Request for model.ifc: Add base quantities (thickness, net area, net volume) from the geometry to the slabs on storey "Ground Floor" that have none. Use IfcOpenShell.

First a look at what the model holds.

```python
import ifcopenshell
import ifcopenshell.util.element
import ifcopenshell.util.unit

model = ifcopenshell.open("model.ifc")
print(model.schema)
for unit_type in ("LENGTHUNIT", "AREAUNIT", "VOLUMEUNIT"):
    print(unit_type, ifcopenshell.util.unit.calculate_unit_scale(model, unit_type))
storey = next(s for s in model.by_type("IfcBuildingStorey") if s.Name == "Ground Floor")
slabs = [e for e in ifcopenshell.util.element.get_decomposition(storey) if e.is_a("IfcSlab")]
for e in sorted(slabs, key=lambda e: e.id()):
    print(e.id(), e.is_a(), e.Name, list(ifcopenshell.util.element.get_psets(e, qtos_only=True)), sep=" | ")
```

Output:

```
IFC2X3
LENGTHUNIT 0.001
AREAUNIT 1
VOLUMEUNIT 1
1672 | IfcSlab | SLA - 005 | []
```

```python
import ifcopenshell
import ifcopenshell.api.pset
import ifcopenshell.geom
import ifcopenshell.util.element
import ifcopenshell.util.shape
import ifcopenshell.util.unit

model = ifcopenshell.open("model.ifc")
unit_scale = ifcopenshell.util.unit.calculate_unit_scale(model)
area_scale = ifcopenshell.util.unit.calculate_unit_scale(model, "AREAUNIT")
volume_scale = ifcopenshell.util.unit.calculate_unit_scale(model, "VOLUMEUNIT")
settings = ifcopenshell.geom.settings()

storey = next(s for s in model.by_type("IfcBuildingStorey") if s.Name == "Ground Floor")
slabs = [e for e in ifcopenshell.util.element.get_decomposition(storey) if e.is_a("IfcSlab")]

for e in sorted(slabs, key=lambda e: e.id()):
    if ifcopenshell.util.element.get_psets(e, qtos_only=True, should_inherit=False):
        continue
    # Geometry comes back in metres, in the element's own axes.
    shape = ifcopenshell.geom.create_shape(settings, e)
    values = {
        "Width": ifcopenshell.util.shape.get_z(shape.geometry) / unit_scale,
        "NetArea": ifcopenshell.util.shape.get_footprint_area(shape.geometry) / area_scale,
        "NetVolume": ifcopenshell.util.shape.get_volume(shape.geometry) / volume_scale,
    }
    qto = ifcopenshell.api.pset.add_qto(model, product=e, name="BaseQuantities")
    ifcopenshell.api.pset.edit_qto(model, qto=qto, properties=values)
    print(e.id(), {k: round(v, 3) for k, v in values.items()})

model.write("model_edited.ifc")
```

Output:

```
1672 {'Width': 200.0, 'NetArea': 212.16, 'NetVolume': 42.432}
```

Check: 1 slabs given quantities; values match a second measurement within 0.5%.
